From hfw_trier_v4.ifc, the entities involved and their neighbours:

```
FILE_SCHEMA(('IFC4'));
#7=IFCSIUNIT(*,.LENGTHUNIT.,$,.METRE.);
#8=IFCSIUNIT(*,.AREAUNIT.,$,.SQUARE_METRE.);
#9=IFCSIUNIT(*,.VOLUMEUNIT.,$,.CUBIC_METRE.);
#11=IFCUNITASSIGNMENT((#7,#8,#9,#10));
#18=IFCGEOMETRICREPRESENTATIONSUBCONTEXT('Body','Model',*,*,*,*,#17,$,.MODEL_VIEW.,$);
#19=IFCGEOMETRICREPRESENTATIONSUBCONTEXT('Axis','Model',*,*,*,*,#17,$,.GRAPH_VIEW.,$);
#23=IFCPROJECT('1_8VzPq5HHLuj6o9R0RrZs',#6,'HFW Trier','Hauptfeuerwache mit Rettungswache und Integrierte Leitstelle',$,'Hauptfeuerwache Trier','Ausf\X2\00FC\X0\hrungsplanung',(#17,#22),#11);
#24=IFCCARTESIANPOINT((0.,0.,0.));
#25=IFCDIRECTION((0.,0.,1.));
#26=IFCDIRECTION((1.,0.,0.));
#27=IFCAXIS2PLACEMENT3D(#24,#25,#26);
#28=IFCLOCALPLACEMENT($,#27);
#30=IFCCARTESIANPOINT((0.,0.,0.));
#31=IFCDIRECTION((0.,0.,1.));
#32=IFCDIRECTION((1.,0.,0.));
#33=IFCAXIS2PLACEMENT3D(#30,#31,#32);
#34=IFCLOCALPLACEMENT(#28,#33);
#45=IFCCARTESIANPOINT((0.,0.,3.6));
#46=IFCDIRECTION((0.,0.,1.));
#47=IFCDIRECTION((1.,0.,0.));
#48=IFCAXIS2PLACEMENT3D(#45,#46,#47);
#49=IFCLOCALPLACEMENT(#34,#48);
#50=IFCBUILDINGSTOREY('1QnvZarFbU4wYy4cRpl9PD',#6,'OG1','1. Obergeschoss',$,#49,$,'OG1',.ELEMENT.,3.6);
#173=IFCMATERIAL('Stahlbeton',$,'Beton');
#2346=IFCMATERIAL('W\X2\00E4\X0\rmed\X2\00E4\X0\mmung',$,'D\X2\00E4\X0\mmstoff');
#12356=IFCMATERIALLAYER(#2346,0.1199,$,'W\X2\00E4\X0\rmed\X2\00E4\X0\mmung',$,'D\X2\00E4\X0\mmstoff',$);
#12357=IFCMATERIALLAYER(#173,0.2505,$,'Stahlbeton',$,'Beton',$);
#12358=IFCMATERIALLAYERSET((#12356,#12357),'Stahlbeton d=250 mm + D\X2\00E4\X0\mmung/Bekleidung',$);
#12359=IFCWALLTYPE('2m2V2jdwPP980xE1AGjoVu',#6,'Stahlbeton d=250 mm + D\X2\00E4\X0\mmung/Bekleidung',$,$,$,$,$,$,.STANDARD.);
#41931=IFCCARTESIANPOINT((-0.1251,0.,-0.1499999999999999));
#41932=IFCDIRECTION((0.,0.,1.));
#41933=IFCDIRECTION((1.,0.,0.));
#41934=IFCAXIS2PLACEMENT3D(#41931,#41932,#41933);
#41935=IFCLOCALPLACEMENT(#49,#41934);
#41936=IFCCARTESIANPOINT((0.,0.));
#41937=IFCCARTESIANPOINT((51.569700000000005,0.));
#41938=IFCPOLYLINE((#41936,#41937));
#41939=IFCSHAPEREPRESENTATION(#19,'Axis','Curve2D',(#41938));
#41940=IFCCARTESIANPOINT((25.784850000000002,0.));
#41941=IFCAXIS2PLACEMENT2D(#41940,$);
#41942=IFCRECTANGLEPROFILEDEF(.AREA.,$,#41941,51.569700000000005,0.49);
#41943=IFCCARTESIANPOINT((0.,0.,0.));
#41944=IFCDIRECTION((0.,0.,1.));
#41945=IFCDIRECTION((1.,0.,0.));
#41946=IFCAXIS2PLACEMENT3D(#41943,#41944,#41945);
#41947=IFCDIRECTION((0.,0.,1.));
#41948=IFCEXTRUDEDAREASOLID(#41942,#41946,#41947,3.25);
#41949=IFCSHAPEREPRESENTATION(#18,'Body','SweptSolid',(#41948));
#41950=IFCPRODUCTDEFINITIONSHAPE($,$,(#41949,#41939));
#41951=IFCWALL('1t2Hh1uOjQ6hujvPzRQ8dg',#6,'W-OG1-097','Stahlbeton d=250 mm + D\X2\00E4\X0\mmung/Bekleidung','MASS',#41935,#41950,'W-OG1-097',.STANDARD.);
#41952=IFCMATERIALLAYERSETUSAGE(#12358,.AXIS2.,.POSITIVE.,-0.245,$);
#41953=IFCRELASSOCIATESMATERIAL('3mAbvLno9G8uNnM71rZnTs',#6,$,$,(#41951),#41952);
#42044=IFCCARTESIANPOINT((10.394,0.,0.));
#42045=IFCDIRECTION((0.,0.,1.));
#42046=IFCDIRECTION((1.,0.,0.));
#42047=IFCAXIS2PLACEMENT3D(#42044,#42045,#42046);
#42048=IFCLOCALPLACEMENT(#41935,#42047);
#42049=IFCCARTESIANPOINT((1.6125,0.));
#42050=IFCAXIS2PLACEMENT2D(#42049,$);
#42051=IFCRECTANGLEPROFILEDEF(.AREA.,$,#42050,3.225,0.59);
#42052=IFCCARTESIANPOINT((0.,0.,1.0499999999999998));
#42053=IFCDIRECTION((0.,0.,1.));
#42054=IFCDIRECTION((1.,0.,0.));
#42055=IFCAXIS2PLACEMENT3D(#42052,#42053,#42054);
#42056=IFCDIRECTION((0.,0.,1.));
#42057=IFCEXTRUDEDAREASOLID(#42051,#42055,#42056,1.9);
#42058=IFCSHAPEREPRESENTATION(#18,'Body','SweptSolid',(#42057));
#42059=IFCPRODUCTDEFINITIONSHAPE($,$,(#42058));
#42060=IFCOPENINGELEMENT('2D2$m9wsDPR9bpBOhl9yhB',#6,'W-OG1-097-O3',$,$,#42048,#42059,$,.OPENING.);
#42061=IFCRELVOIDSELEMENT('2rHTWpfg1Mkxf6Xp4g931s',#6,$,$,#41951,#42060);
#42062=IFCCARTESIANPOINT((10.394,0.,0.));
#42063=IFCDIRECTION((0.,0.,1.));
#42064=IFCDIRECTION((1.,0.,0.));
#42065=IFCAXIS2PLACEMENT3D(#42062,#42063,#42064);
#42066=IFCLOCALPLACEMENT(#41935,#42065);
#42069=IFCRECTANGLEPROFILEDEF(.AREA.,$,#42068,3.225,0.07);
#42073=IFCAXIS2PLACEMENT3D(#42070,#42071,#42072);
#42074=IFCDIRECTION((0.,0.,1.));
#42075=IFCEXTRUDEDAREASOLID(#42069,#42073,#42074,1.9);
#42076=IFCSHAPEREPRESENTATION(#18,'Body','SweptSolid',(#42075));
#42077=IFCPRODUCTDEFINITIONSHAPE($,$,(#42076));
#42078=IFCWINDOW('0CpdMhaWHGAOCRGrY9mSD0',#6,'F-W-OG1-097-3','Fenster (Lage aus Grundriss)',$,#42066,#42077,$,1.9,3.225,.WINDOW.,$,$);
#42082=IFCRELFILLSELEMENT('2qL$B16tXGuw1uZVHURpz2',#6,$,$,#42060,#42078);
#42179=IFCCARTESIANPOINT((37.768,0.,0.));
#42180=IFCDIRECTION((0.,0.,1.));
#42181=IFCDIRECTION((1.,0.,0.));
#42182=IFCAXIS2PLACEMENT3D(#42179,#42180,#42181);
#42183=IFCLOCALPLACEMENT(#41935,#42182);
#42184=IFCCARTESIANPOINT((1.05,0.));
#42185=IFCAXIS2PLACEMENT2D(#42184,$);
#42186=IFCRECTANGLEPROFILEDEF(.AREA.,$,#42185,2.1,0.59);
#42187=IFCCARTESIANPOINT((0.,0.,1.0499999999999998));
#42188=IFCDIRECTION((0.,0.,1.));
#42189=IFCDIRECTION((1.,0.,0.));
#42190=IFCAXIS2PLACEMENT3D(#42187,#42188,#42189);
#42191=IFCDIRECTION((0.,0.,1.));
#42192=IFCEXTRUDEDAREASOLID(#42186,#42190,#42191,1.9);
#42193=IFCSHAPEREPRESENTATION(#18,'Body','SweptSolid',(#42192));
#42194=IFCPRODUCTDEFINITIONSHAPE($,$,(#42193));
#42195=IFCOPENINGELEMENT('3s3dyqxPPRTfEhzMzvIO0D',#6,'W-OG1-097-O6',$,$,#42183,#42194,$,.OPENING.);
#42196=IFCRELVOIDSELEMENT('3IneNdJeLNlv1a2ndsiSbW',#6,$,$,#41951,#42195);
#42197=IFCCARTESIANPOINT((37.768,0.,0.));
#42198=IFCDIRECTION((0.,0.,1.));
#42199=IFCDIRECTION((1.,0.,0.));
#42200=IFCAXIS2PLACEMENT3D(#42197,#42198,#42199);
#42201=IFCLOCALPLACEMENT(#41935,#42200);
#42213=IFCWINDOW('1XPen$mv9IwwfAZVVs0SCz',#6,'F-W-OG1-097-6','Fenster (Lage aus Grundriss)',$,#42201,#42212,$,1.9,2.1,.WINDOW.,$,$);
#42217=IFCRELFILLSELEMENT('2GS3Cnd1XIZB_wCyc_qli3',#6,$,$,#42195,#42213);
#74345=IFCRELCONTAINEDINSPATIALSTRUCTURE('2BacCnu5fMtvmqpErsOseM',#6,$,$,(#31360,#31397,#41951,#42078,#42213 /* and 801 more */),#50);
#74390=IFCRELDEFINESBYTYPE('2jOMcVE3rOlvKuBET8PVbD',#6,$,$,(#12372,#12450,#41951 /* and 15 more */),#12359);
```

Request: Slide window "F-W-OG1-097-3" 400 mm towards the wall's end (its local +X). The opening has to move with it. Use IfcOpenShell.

```python
import ifcopenshell
import ifcopenshell.api.geometry
import ifcopenshell.util.placement
import ifcopenshell.util.unit

model = ifcopenshell.open("hfw_trier_v4.ifc")
unit_scale = ifcopenshell.util.unit.calculate_unit_scale(model)

window = model.by_id(42078)
opening = window.FillsVoids[0].RelatingOpeningElement
wall = opening.VoidsElements[0].RelatingBuildingElement

wall_matrix = ifcopenshell.util.placement.get_local_placement(wall.ObjectPlacement)
shift = wall_matrix[:3, 0] * 0.4 / unit_scale
before = ifcopenshell.util.placement.get_local_placement(window.ObjectPlacement)[:3, 3].copy()

# The window is not placed relative to its opening, so move both.
for product in (opening, window):
    matrix = ifcopenshell.util.placement.get_local_placement(product.ObjectPlacement)
    matrix[:3, 3] += shift
    ifcopenshell.api.geometry.edit_object_placement(model, product=product, matrix=matrix, is_si=False)

after = ifcopenshell.util.placement.get_local_placement(window.ObjectPlacement)[:3, 3]
print("window moved by", (after - before).round(3) + 0.0)

model.write("hfw_trier_v4-out.ifc")
```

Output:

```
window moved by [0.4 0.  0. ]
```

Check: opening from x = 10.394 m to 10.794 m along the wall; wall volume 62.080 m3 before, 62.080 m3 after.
